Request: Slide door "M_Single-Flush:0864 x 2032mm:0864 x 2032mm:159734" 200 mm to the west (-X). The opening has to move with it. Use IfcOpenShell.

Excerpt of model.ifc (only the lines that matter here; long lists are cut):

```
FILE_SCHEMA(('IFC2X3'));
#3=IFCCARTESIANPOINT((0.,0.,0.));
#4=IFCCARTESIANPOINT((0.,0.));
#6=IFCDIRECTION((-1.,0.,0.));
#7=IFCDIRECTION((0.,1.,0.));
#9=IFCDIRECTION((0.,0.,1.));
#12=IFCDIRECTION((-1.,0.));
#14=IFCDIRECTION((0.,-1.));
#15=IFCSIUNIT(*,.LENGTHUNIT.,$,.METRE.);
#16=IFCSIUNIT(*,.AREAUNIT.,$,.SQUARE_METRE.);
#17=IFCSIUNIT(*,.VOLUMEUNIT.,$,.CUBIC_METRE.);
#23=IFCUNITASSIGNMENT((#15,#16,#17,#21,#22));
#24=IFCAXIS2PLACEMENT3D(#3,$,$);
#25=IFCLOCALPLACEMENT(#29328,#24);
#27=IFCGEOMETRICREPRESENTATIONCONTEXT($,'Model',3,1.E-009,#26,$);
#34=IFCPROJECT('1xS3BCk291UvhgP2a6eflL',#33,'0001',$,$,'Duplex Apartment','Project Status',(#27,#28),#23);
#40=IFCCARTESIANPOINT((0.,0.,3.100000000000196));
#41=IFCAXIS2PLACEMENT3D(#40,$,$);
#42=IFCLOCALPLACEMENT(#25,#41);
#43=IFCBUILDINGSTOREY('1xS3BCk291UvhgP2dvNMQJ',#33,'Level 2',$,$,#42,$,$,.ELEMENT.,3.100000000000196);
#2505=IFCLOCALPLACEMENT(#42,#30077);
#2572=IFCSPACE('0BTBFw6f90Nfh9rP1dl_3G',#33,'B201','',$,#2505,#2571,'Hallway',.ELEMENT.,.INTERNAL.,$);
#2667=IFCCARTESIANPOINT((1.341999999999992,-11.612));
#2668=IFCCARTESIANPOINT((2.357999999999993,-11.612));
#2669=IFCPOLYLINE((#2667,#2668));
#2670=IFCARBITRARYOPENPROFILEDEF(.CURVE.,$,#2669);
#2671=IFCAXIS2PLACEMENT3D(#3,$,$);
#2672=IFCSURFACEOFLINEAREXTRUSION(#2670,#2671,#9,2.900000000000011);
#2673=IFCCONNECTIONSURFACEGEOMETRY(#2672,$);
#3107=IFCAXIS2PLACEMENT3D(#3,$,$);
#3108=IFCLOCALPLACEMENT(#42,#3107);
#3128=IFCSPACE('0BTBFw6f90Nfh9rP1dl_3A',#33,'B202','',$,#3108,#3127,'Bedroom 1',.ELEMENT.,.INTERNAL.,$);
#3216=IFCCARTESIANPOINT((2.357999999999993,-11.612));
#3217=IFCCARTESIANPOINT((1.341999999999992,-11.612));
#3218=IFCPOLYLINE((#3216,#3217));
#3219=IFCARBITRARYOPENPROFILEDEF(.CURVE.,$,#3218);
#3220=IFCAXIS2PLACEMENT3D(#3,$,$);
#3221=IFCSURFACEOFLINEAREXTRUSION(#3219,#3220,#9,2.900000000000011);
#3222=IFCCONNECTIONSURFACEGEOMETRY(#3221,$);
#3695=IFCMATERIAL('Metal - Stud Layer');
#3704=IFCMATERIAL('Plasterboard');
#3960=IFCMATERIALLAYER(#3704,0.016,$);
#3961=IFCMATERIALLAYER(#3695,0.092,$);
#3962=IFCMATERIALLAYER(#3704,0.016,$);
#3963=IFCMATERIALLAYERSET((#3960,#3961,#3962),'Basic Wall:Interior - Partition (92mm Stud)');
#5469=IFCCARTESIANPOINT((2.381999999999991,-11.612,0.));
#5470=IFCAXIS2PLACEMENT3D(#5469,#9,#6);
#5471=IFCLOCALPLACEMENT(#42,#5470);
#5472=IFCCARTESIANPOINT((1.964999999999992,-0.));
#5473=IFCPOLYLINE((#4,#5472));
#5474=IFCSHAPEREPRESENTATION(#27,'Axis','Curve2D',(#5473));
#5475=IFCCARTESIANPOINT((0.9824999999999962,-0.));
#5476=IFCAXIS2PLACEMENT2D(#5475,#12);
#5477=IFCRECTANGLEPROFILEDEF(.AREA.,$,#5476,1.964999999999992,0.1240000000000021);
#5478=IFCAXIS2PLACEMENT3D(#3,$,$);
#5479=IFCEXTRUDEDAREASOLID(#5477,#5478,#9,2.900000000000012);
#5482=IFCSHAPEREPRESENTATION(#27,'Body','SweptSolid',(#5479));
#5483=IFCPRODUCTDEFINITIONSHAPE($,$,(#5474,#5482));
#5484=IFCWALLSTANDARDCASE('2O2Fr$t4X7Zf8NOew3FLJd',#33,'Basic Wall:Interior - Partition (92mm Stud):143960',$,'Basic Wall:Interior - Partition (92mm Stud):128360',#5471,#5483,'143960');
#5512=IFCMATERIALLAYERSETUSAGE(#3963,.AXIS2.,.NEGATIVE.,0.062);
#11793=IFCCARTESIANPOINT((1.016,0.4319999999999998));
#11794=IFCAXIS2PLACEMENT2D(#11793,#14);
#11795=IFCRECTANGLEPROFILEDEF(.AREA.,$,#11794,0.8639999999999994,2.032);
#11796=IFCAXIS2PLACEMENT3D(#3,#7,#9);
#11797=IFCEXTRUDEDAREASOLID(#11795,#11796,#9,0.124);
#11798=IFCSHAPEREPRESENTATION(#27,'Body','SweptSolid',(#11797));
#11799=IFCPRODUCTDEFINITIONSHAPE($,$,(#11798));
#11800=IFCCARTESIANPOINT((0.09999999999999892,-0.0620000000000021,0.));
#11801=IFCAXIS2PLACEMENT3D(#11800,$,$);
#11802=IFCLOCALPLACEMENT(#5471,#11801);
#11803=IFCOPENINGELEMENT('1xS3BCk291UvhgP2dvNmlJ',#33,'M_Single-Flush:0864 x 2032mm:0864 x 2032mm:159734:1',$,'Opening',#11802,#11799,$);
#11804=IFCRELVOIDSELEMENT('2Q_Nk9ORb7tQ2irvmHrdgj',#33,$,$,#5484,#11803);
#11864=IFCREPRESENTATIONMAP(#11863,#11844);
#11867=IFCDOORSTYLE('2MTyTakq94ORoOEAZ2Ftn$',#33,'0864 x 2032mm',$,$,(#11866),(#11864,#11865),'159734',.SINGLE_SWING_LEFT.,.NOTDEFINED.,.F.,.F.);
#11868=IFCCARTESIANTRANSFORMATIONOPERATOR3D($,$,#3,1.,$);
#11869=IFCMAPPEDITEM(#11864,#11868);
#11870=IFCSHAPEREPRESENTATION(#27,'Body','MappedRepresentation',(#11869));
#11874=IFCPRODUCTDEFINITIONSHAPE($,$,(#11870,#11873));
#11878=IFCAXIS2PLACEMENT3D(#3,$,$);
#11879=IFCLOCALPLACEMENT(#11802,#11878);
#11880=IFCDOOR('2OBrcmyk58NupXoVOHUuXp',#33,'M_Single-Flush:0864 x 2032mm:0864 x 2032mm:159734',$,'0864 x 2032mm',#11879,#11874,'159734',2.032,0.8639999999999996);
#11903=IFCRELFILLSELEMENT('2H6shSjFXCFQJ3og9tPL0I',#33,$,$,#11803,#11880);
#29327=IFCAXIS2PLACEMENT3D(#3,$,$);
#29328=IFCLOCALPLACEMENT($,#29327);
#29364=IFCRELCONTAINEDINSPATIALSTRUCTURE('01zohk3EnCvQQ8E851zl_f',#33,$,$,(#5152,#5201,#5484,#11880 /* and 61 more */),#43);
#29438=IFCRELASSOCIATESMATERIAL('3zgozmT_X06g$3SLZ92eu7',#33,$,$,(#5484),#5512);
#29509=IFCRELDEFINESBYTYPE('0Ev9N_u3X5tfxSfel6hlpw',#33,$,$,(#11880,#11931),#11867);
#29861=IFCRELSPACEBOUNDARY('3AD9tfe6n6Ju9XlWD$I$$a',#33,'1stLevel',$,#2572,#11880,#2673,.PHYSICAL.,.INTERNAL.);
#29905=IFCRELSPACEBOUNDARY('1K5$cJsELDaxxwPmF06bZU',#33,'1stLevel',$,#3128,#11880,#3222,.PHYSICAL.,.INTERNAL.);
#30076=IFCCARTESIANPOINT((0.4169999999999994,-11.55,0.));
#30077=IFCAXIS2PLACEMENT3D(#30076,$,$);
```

```python
import numpy as np
import ifcopenshell
import ifcopenshell.api.geometry
import ifcopenshell.util.placement
import ifcopenshell.util.unit

model = ifcopenshell.open("model.ifc")
unit_scale = ifcopenshell.util.unit.calculate_unit_scale(model)

door = model.by_id(11880)
opening = door.FillsVoids[0].RelatingOpeningElement
wall = opening.VoidsElements[0].RelatingBuildingElement

wall_matrix = ifcopenshell.util.placement.get_local_placement(wall.ObjectPlacement)
shift = wall_matrix[:3, 0] * 0.2 / unit_scale
before = ifcopenshell.util.placement.get_local_placement(door.ObjectPlacement)[:3, 3].copy()

# The door is placed relative to its opening, so it follows when the opening moves.
matrix = ifcopenshell.util.placement.get_local_placement(opening.ObjectPlacement)
matrix[:3, 3] += shift
ifcopenshell.api.geometry.edit_object_placement(
    model, product=opening, matrix=matrix, is_si=False, should_transform_children=True
)

# Space boundary surfaces are stored in each space's coordinates; move them too.
for rel in door.ProvidesBoundaries:
    if not rel.ConnectionGeometry:
        continue
    surface = rel.ConnectionGeometry.SurfaceOnRelatingElement
    space_matrix = ifcopenshell.util.placement.get_local_placement(rel.RelatingSpace.ObjectPlacement)
    point = np.array(surface.Position.Location.Coordinates) + space_matrix[:3, :3].T @ shift
    surface.Position = model.createIfcAxis2Placement3D(
        model.createIfcCartesianPoint(point.tolist()), surface.Position.Axis, surface.Position.RefDirection
    )

after = ifcopenshell.util.placement.get_local_placement(door.ObjectPlacement)[:3, 3]
print("door moved by", (after - before).round(3) + 0.0)

model.write("model_rev.ifc")
```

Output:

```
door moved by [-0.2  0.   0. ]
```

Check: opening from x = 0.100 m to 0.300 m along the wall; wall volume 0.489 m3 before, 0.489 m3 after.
